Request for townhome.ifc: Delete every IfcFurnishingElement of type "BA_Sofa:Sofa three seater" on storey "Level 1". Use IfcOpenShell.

First a look at what the model holds.

```python
import ifcopenshell
import ifcopenshell.util.element

model = ifcopenshell.open("townhome.ifc")
print(model.schema)
storey = next(s for s in model.by_type("IfcBuildingStorey") if s.Name == "Level 1")
furniture = [e for e in ifcopenshell.util.element.get_decomposition(storey) if e.is_a("IfcFurnishingElement")]
seen = {}
for e in furniture:
    element_type = ifcopenshell.util.element.get_type(e)
    name = element_type.Name if element_type not in (None, e) else None
    seen[name] = seen.get(name, 0) + 1
for name, count in sorted(seen.items(), key=str):
    print(count, "x", name)
```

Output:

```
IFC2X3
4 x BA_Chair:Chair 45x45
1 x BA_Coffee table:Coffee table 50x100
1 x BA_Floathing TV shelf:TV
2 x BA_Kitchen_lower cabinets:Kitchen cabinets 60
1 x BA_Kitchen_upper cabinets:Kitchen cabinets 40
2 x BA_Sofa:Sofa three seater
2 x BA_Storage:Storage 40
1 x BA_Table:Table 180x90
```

```python
import ifcopenshell
import ifcopenshell.api.root
import ifcopenshell.util.element

model = ifcopenshell.open("townhome.ifc")

storey = next(s for s in model.by_type("IfcBuildingStorey") if s.Name == "Level 1")
furniture = [e for e in ifcopenshell.util.element.get_decomposition(storey) if e.is_a("IfcFurnishingElement")]
targets = [e for e in furniture if (t := ifcopenshell.util.element.get_type(e)) not in (None, e) and t.Name == "BA_Sofa:Sofa three seater"]

for e in targets:
    ifcopenshell.api.root.remove_product(model, product=e)
print(len(targets), "removed")

model.write("townhome-out.ifc")
```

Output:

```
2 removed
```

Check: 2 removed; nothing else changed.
